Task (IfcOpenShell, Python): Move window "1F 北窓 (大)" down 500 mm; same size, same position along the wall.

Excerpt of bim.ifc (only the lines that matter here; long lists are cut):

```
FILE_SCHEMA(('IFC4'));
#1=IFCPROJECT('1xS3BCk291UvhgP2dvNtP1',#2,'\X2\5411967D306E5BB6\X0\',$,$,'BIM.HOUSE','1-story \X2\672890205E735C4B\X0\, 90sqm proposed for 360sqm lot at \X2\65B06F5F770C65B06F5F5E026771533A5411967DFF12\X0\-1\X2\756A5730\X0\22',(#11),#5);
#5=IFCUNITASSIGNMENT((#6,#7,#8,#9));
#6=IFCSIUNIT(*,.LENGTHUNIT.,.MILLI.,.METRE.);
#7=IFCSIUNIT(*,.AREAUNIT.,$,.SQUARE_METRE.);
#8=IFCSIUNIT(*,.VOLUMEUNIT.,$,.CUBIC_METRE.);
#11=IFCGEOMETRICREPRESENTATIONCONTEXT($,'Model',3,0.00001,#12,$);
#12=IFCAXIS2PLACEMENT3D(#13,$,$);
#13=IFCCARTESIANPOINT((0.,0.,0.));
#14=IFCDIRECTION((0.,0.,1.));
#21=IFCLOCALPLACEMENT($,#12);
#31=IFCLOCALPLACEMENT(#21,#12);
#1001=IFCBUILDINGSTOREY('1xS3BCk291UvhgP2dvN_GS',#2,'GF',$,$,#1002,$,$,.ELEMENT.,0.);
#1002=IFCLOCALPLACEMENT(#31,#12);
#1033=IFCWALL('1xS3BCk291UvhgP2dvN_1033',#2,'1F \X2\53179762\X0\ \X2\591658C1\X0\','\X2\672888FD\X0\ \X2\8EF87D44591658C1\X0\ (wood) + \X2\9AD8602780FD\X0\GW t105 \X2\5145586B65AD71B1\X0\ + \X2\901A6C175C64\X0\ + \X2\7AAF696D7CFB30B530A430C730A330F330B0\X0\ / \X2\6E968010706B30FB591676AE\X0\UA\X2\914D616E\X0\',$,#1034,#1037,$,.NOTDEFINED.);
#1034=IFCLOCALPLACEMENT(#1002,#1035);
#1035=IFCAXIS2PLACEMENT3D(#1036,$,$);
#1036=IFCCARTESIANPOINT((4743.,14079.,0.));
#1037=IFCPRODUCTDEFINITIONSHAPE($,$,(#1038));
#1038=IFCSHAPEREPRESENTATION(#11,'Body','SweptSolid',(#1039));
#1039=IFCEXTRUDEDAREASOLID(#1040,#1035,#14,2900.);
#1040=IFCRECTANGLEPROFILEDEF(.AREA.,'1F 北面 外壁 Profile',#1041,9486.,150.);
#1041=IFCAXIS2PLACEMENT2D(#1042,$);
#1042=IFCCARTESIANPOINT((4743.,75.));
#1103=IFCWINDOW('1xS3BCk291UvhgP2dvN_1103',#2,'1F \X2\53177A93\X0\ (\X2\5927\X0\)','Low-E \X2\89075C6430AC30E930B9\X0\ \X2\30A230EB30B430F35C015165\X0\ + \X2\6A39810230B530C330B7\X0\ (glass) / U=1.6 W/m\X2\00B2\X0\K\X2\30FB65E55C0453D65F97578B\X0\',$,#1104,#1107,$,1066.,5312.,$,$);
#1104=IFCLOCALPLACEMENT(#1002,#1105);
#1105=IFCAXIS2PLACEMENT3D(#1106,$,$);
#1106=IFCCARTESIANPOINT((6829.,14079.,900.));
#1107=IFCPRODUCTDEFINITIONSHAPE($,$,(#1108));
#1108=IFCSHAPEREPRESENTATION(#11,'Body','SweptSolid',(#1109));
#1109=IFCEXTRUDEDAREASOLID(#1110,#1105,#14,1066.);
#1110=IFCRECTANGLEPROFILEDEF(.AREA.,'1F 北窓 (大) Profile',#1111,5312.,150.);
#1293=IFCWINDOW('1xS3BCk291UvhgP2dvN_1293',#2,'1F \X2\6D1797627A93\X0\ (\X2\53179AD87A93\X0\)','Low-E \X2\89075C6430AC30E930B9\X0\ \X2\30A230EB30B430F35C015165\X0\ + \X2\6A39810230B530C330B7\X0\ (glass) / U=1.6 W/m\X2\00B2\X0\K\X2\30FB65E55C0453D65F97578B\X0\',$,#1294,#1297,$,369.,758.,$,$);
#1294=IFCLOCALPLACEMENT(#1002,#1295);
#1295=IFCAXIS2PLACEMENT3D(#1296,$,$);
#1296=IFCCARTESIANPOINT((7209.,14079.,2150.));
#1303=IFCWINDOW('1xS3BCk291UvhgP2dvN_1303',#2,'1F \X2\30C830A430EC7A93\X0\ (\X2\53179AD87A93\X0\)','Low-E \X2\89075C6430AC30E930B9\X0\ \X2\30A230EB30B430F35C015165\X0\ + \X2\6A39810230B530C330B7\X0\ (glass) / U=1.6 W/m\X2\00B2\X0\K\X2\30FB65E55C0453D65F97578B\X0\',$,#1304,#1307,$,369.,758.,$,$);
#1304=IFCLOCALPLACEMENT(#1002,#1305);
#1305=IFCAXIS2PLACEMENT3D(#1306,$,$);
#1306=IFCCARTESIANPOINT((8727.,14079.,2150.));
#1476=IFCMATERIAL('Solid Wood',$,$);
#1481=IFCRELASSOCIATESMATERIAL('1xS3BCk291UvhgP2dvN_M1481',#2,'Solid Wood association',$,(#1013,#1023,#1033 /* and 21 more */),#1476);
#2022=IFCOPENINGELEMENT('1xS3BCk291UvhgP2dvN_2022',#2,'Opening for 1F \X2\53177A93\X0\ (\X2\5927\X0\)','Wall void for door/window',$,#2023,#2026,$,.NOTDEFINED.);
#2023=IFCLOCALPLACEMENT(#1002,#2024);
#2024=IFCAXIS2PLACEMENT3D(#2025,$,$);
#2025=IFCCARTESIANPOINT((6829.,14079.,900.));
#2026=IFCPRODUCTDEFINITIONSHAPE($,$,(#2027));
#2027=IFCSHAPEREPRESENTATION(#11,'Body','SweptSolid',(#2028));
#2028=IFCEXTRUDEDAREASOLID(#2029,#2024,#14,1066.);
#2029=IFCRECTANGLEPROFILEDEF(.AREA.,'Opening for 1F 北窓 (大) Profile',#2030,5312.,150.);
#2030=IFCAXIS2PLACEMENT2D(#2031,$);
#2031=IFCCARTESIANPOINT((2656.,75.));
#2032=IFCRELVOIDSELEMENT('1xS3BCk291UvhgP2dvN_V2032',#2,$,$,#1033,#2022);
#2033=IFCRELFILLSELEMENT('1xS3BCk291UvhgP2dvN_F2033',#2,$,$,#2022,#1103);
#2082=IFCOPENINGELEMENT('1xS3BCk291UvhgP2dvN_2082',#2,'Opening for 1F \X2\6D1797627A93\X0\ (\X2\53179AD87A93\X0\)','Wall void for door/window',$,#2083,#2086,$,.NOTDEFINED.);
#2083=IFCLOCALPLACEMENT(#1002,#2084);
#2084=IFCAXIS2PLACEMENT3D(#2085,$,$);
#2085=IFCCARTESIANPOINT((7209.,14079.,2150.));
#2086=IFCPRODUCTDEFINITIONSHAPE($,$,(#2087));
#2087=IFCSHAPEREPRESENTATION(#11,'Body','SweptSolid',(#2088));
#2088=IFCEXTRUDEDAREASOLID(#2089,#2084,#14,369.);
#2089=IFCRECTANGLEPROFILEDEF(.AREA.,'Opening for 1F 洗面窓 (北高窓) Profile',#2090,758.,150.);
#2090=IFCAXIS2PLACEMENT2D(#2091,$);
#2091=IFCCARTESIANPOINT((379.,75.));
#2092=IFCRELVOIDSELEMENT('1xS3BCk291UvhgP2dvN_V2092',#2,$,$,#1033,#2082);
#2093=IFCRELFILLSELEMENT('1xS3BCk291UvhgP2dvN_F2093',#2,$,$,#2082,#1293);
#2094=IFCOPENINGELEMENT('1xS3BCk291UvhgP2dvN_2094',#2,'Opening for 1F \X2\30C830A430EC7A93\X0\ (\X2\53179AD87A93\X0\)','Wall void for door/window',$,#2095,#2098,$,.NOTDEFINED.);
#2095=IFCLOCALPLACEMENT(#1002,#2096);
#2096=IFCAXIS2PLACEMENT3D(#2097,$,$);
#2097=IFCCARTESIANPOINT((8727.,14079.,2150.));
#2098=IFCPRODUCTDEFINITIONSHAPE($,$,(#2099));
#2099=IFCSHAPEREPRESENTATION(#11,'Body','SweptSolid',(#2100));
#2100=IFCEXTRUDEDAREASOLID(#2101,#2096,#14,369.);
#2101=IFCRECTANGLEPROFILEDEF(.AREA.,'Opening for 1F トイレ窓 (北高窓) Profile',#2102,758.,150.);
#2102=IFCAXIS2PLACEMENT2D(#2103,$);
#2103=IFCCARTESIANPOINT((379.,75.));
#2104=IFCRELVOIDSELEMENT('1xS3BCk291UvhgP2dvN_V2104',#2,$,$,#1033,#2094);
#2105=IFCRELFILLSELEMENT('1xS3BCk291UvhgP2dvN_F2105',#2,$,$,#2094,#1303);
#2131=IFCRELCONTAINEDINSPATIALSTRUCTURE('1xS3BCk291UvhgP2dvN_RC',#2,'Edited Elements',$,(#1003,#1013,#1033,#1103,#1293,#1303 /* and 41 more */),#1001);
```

```python
import numpy as np
import ifcopenshell
import ifcopenshell.api.geometry
import ifcopenshell.util.placement
import ifcopenshell.util.unit

model = ifcopenshell.open("bim.ifc")
unit_scale = ifcopenshell.util.unit.calculate_unit_scale(model)

window = model.by_guid("1xS3BCk291UvhgP2dvN_1103")
opening = window.FillsVoids[0].RelatingOpeningElement
dz = -0.5 / unit_scale

shift = np.array([0.0, 0.0, dz])
# The window is not placed relative to its opening, so move both.
for product in (opening, window):
    matrix = ifcopenshell.util.placement.get_local_placement(product.ObjectPlacement)
    matrix[:3, 3] += shift
    ifcopenshell.api.geometry.edit_object_placement(model, product=product, matrix=matrix, is_si=False)

print(f"moved by {dz * unit_scale:+.3f} m")

model.write("bim_rev.ifc")
```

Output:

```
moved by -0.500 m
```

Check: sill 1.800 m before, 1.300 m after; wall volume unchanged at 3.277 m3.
